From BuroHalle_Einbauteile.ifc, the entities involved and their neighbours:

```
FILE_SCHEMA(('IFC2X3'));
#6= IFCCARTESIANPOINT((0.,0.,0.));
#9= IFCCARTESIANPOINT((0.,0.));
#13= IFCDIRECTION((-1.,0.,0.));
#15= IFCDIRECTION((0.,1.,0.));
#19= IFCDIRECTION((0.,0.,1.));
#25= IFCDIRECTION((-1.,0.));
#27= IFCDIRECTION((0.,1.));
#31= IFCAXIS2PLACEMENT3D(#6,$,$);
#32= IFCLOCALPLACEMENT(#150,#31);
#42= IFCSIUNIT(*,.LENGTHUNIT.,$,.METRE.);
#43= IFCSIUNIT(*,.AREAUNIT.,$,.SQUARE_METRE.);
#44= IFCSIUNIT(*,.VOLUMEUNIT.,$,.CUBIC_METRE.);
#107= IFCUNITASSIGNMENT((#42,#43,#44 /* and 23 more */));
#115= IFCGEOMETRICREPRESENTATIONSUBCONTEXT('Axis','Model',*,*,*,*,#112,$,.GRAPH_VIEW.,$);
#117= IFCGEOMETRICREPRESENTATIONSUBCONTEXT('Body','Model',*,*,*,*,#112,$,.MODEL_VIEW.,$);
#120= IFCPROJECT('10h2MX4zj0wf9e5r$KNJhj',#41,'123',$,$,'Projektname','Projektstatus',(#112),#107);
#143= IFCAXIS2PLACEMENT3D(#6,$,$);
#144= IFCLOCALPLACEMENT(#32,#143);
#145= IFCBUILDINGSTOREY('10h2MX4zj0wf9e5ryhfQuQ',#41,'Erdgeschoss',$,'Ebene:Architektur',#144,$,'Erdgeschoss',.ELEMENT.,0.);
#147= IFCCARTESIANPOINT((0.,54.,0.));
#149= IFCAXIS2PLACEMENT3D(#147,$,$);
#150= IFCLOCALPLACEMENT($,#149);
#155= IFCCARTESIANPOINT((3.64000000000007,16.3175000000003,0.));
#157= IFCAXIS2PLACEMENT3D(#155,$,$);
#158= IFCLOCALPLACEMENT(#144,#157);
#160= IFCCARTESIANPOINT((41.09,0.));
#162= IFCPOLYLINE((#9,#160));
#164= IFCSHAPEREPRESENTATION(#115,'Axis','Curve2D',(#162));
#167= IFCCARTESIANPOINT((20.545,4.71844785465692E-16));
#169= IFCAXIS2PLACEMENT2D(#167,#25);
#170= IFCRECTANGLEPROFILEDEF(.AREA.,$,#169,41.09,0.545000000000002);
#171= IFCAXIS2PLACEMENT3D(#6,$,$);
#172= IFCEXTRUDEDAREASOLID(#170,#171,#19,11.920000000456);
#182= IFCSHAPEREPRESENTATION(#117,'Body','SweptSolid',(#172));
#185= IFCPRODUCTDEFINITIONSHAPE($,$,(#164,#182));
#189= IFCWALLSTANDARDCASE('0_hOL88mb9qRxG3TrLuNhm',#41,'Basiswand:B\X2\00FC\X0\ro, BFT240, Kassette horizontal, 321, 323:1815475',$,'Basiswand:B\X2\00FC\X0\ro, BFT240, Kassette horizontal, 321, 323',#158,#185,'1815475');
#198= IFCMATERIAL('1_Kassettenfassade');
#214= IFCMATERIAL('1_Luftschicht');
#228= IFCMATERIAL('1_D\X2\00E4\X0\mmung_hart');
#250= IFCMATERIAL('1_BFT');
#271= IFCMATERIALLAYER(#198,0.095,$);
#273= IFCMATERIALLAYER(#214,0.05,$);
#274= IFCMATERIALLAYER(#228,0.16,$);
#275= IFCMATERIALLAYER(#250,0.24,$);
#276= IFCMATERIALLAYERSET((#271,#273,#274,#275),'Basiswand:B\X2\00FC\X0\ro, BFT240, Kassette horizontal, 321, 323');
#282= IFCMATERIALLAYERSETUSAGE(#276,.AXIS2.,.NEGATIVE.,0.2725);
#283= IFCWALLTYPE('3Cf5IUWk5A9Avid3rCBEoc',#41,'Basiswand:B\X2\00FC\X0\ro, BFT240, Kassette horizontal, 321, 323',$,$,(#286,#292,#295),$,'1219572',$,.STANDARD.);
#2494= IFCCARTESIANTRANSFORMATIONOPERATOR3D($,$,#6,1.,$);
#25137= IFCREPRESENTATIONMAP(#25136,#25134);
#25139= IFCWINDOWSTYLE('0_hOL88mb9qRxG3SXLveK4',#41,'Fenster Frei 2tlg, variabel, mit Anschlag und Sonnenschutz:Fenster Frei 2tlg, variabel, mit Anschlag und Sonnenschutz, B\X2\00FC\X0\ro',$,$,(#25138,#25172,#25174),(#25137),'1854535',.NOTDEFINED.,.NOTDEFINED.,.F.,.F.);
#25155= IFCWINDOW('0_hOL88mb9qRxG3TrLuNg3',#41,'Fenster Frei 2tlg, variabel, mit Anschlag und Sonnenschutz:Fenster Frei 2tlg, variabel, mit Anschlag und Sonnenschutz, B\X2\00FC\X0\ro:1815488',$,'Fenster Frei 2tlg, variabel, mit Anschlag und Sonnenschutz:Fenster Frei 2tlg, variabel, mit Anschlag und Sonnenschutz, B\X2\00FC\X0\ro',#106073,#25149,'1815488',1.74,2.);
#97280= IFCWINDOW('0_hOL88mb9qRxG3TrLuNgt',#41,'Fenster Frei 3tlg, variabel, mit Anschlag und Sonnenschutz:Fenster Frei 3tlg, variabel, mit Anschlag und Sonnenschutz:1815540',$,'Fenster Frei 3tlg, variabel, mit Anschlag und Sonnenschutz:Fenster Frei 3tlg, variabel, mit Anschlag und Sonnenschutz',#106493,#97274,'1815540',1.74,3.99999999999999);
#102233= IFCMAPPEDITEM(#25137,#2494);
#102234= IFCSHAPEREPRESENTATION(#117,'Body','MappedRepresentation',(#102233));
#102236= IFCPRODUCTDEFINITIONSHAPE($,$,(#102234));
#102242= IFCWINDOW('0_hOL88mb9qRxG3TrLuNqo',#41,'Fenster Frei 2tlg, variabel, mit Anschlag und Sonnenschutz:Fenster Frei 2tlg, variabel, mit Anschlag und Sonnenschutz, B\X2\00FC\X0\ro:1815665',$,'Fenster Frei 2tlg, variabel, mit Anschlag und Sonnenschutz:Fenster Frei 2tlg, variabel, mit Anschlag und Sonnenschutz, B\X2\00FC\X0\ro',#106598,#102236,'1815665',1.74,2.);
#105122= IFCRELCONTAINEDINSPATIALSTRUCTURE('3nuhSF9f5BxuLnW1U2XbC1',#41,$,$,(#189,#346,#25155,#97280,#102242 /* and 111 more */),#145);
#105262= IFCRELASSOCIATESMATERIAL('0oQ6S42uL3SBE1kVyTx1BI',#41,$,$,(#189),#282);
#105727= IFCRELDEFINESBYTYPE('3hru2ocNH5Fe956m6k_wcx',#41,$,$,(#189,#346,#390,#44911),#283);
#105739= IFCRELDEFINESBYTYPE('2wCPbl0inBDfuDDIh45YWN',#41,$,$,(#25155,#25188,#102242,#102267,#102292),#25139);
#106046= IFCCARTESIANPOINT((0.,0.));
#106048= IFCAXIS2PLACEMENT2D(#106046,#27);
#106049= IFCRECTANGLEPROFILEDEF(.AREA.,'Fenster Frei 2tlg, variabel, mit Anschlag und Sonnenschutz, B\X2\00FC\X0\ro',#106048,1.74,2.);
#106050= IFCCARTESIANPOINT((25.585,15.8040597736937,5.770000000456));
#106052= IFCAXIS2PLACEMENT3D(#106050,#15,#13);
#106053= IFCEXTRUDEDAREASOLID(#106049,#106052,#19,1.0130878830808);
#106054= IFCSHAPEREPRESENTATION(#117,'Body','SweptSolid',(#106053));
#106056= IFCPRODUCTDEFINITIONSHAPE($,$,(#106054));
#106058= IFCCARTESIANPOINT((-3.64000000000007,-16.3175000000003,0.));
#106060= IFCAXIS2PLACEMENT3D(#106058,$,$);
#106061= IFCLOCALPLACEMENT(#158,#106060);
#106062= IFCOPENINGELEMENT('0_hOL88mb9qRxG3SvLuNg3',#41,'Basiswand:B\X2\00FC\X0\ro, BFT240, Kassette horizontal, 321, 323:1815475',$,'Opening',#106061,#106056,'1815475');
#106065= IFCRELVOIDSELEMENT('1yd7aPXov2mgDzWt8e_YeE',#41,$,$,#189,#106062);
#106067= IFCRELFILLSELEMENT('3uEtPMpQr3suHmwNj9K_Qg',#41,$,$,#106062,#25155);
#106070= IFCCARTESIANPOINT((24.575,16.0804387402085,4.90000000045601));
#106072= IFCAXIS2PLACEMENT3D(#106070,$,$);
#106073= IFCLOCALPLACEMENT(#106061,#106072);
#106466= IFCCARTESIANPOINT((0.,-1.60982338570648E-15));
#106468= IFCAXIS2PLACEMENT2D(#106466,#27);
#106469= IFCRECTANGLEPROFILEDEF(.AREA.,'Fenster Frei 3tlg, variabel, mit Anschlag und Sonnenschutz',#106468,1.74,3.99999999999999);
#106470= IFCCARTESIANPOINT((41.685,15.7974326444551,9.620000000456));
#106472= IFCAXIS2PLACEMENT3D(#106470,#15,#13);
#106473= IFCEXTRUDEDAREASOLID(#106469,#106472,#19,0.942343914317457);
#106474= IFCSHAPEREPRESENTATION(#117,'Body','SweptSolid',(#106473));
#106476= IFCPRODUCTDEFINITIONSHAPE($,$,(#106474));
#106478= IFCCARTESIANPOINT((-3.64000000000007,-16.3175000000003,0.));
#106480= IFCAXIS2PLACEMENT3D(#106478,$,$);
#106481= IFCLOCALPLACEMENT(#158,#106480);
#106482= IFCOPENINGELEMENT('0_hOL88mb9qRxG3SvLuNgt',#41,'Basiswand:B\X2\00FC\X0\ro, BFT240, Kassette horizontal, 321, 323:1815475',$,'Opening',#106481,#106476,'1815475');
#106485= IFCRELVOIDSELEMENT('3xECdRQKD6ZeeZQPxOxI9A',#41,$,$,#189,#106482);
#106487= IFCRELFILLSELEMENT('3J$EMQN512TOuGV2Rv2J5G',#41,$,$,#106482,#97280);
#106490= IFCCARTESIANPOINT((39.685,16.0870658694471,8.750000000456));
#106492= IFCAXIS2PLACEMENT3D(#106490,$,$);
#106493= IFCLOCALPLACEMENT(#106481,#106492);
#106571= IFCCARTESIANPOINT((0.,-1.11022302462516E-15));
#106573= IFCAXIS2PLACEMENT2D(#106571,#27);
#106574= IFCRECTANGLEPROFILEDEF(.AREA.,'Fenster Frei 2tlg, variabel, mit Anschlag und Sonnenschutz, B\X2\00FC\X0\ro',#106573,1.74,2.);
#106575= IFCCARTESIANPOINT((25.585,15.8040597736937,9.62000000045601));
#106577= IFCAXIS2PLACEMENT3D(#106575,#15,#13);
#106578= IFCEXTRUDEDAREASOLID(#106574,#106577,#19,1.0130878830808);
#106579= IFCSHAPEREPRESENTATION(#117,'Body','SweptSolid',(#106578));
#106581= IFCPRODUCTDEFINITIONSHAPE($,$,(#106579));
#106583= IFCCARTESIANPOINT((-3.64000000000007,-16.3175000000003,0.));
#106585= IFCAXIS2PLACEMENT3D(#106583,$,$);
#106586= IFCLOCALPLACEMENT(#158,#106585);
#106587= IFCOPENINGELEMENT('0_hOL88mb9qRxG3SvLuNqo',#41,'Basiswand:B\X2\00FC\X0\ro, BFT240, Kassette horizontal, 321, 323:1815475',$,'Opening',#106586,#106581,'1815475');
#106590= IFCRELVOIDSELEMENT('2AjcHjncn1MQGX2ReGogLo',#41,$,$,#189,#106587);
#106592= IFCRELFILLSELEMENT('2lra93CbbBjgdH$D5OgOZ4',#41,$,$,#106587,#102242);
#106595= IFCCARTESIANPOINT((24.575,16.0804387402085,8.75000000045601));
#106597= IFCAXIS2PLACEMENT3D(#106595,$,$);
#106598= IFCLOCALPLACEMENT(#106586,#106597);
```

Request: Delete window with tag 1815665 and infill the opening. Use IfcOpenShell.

```python
import ifcopenshell
import ifcopenshell.api.feature
import ifcopenshell.api.root
import ifcopenshell.geom
import ifcopenshell.util.shape

model = ifcopenshell.open("BuroHalle_Einbauteile.ifc")
settings = ifcopenshell.geom.settings()


def volume(element):
    """Net volume in cubic metres, openings subtracted."""
    shape = ifcopenshell.geom.create_shape(settings, element)
    return ifcopenshell.util.shape.get_volume(shape.geometry)


window = model.by_id(102242)
opening = window.FillsVoids[0].RelatingOpeningElement
wall = opening.VoidsElements[0].RelatingBuildingElement
before = volume(wall)

ifcopenshell.api.root.remove_product(model, product=window)
ifcopenshell.api.feature.remove_feature(model, feature=opening)

after = volume(wall)

print(f"wall volume {before:.3f} -> {after:.3f} m3")

model.write("BuroHalle_Einbauteile_edited.ifc")
```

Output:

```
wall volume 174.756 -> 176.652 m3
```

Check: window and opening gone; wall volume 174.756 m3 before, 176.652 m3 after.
